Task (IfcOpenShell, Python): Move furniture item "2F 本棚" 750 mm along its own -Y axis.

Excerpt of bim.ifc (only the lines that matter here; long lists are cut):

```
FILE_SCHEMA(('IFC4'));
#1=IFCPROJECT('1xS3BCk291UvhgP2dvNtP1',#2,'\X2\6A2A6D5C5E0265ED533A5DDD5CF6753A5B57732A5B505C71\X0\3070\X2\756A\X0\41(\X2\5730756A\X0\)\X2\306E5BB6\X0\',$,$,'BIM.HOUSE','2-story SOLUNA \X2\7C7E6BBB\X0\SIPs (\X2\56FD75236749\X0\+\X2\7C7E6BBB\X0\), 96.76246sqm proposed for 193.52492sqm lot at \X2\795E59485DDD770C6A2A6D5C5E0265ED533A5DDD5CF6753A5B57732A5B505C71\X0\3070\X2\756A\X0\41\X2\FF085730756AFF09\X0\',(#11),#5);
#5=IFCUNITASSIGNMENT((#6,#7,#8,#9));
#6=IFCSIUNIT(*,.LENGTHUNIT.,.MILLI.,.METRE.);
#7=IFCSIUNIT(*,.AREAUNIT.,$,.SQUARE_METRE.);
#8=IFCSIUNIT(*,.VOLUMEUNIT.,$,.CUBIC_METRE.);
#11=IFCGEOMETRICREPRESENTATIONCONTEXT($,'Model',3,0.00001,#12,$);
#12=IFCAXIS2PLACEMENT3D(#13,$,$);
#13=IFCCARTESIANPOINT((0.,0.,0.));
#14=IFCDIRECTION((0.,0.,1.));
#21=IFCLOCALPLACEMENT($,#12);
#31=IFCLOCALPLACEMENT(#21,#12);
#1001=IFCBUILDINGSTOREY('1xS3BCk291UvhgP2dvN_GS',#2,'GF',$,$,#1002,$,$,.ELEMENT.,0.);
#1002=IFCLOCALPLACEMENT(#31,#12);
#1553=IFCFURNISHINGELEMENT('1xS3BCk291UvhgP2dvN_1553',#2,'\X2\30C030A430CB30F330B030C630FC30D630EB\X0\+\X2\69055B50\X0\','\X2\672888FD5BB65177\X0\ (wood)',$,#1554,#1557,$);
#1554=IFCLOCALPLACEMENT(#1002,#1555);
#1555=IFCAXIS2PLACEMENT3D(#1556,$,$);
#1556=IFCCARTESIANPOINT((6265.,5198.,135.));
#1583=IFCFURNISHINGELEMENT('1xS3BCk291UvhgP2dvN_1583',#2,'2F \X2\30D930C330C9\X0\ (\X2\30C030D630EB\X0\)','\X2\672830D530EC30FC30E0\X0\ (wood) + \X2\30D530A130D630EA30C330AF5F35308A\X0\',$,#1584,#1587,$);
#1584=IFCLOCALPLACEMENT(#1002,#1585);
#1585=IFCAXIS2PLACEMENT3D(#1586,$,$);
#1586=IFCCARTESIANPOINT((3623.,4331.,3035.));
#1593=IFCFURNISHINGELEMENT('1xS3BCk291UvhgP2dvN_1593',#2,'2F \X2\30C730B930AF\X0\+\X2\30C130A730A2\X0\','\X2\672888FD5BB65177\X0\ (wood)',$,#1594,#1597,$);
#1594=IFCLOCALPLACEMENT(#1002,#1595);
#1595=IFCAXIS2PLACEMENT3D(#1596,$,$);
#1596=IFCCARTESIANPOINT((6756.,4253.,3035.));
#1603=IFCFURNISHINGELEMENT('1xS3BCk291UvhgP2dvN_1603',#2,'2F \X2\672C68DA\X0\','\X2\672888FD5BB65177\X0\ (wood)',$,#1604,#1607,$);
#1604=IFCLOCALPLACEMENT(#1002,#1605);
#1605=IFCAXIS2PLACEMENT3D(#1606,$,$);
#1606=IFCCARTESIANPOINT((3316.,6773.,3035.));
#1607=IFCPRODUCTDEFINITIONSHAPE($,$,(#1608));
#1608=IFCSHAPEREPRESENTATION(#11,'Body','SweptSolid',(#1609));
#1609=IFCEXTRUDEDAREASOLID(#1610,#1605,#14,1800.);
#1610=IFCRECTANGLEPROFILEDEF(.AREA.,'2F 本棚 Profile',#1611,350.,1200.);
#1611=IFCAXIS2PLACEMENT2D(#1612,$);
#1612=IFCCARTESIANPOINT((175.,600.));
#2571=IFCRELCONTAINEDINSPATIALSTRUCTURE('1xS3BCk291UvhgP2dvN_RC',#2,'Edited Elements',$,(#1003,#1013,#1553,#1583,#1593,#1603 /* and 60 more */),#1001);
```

```python
import ifcopenshell
import ifcopenshell.api.geometry
import ifcopenshell.util.placement
import ifcopenshell.util.unit

model = ifcopenshell.open("bim.ifc")
unit_scale = ifcopenshell.util.unit.calculate_unit_scale(model)

item = model.by_id(1603)
matrix = ifcopenshell.util.placement.get_local_placement(item.ObjectPlacement)
matrix[:3, 3] -= matrix[:3, 1] * 0.75 / unit_scale
ifcopenshell.api.geometry.edit_object_placement(model, product=item, matrix=matrix, is_si=False)

print(ifcopenshell.util.placement.get_local_placement(item.ObjectPlacement).round(3) + 0.0)

model.write("bim_rev.ifc")
```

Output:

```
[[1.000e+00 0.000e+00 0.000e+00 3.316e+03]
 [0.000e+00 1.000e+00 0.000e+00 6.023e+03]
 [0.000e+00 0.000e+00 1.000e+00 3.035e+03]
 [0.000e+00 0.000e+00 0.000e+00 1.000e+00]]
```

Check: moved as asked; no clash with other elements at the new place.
